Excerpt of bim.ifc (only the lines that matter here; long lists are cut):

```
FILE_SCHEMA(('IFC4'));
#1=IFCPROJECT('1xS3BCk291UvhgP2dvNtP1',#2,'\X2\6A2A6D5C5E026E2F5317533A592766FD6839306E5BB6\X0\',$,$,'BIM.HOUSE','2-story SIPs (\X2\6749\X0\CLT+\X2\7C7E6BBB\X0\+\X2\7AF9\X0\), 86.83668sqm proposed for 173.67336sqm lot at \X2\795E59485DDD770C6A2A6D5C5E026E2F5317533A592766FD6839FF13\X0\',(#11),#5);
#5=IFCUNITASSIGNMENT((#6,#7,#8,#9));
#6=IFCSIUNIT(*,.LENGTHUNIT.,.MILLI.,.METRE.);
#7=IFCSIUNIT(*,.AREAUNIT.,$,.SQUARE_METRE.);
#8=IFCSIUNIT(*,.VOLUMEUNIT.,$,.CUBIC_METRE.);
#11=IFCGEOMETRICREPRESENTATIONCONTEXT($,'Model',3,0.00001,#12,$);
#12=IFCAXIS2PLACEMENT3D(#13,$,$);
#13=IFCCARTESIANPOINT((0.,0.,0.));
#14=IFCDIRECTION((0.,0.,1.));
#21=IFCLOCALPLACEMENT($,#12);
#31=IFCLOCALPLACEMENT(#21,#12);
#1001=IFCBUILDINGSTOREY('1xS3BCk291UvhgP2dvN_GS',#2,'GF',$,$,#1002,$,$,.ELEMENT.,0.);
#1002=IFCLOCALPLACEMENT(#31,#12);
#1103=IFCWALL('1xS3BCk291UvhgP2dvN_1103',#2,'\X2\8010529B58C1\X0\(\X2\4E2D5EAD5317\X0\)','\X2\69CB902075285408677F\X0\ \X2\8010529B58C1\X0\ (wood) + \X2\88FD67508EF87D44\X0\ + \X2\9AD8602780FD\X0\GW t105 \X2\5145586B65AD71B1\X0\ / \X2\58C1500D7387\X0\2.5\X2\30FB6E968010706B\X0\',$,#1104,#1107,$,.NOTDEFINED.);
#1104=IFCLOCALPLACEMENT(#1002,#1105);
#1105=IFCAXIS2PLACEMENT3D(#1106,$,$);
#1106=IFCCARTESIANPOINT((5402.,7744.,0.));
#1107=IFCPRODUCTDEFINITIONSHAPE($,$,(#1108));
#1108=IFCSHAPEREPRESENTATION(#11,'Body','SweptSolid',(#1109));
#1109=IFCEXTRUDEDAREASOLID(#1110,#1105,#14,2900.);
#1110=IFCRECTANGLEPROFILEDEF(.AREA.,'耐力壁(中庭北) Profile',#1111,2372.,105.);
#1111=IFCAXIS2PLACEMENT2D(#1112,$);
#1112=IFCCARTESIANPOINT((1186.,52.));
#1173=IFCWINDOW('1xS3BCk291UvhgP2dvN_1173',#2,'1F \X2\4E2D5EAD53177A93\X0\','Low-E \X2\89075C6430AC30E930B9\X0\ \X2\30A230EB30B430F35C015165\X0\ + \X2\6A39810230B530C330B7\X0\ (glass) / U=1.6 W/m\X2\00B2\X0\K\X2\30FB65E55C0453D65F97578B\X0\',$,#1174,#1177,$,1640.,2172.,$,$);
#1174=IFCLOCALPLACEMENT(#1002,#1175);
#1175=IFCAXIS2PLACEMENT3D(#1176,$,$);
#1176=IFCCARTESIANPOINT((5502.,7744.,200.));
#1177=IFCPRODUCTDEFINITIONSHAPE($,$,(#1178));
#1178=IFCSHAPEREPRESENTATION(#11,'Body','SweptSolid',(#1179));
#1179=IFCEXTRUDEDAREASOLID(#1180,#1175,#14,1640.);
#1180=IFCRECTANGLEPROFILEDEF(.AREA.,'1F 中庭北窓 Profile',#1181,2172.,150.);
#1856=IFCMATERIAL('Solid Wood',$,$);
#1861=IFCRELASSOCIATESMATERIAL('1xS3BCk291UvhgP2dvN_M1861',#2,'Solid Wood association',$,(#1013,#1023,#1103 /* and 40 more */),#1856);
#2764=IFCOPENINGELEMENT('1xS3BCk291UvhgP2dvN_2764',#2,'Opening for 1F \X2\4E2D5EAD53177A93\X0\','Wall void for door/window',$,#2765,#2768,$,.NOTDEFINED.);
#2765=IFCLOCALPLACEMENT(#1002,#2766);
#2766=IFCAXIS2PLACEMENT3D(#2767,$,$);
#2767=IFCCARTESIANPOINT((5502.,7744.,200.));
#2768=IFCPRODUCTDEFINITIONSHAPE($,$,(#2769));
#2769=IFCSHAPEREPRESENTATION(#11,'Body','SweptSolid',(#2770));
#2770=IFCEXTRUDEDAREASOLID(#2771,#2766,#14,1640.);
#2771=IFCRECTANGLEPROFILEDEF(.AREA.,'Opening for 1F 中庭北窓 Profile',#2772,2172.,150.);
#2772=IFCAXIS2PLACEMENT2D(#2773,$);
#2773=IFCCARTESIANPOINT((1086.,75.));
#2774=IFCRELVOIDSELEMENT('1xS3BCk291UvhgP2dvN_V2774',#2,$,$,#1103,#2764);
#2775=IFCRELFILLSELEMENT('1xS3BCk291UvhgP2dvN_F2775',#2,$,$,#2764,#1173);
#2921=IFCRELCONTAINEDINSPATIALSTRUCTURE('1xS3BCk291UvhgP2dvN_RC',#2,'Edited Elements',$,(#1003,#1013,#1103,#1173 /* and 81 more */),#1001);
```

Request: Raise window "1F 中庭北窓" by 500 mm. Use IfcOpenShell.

```python
import numpy as np
import ifcopenshell
import ifcopenshell.api.geometry
import ifcopenshell.util.placement
import ifcopenshell.util.unit

model = ifcopenshell.open("bim.ifc")
unit_scale = ifcopenshell.util.unit.calculate_unit_scale(model)

window = model.by_id(1173)
opening = window.FillsVoids[0].RelatingOpeningElement
dz = 500.0

shift = np.array([0.0, 0.0, dz])
# The window is not placed relative to its opening, so move both.
for product in (opening, window):
    matrix = ifcopenshell.util.placement.get_local_placement(product.ObjectPlacement)
    matrix[:3, 3] += shift
    ifcopenshell.api.geometry.edit_object_placement(model, product=product, matrix=matrix, is_si=False)

print(f"moved by {dz * unit_scale:+.3f} m")

model.write("bim_edited.ifc")
```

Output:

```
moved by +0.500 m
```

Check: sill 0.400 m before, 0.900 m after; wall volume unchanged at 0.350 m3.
